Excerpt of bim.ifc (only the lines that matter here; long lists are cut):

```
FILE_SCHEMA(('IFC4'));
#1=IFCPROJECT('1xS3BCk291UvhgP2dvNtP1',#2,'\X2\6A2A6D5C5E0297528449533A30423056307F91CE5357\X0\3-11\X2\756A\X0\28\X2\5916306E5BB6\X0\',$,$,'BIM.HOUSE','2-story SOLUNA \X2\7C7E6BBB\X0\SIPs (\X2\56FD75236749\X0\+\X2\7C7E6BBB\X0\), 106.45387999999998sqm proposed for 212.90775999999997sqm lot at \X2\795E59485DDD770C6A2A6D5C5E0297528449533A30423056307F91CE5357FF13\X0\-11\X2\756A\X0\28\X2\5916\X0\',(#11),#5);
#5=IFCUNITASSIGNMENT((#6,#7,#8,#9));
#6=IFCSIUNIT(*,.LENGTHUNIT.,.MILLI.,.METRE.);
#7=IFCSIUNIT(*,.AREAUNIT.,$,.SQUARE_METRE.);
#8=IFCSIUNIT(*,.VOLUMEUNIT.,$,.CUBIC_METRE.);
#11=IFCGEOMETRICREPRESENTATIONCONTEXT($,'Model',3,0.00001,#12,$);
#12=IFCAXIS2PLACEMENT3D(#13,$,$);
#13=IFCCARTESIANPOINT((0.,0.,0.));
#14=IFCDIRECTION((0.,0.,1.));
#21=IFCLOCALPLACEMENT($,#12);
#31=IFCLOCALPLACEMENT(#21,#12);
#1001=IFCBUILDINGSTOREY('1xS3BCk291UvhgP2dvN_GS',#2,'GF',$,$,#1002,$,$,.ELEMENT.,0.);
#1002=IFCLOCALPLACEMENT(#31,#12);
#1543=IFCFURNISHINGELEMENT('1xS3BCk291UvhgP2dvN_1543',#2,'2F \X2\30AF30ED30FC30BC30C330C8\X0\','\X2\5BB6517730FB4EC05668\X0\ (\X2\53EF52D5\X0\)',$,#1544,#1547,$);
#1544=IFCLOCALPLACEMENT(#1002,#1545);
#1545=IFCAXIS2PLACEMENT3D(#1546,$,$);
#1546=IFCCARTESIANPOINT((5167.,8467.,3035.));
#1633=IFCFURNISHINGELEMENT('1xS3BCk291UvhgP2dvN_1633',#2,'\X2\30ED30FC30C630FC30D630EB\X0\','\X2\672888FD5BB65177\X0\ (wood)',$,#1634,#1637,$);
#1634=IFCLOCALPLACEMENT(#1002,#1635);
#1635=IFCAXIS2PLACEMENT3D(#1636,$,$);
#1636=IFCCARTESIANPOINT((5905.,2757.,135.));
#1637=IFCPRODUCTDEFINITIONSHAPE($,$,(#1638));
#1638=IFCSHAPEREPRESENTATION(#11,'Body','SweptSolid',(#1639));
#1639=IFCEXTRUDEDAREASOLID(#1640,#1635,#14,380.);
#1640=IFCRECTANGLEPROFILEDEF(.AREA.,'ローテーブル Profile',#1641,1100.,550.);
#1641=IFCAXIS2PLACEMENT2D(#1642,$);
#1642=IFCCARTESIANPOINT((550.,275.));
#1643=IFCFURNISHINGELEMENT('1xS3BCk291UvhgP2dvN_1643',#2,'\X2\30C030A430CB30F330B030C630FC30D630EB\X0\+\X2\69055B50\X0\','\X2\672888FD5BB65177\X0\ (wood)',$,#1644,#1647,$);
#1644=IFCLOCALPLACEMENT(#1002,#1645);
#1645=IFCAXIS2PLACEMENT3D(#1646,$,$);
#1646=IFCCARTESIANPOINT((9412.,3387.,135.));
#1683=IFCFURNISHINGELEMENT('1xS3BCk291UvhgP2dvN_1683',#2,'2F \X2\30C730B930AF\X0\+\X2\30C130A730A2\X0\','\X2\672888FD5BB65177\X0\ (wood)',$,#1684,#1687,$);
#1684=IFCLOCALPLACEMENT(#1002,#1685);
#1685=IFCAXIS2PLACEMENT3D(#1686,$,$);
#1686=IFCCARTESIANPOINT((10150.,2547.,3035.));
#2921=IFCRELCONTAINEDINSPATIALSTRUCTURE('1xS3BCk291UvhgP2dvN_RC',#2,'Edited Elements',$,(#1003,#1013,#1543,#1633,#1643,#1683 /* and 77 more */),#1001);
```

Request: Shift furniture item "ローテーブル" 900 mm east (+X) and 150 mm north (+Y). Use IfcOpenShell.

```python
import ifcopenshell
import ifcopenshell.api.geometry
import ifcopenshell.util.placement
import ifcopenshell.util.unit

model = ifcopenshell.open("bim.ifc")
unit_scale = ifcopenshell.util.unit.calculate_unit_scale(model)

item = model.by_guid("1xS3BCk291UvhgP2dvN_1633")
matrix = ifcopenshell.util.placement.get_local_placement(item.ObjectPlacement)
matrix[0, 3] += 0.9 / unit_scale
matrix[1, 3] += 0.15 / unit_scale
ifcopenshell.api.geometry.edit_object_placement(model, product=item, matrix=matrix, is_si=False)

print(ifcopenshell.util.placement.get_local_placement(item.ObjectPlacement).round(3) + 0.0)

model.write("bim_updated.ifc")
```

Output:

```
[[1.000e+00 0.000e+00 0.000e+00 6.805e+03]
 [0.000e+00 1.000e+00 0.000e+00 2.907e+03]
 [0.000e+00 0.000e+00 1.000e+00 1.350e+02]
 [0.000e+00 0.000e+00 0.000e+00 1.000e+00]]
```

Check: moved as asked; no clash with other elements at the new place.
